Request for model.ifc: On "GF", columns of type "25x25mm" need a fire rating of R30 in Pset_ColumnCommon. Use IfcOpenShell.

First a look at what the model holds.

```python
import ifcopenshell
import ifcopenshell.util.element

model = ifcopenshell.open("model.ifc")
print(model.schema)
storey = next(s for s in model.by_type("IfcBuildingStorey") if s.Name == "GF")
columns = [e for e in ifcopenshell.util.element.get_decomposition(storey) if e.is_a("IfcColumn")]
seen = {}
for e in columns:
    element_type = ifcopenshell.util.element.get_type(e)
    key = (element_type.Name if element_type != e and element_type else None, ifcopenshell.util.element.get_pset(e, "Pset_ColumnCommon", "FireRating"))
    seen[key] = seen.get(key, 0) + 1
for (name, value), count in sorted(seen.items(), key=str):
    print(count, "x", name, "|", value)
```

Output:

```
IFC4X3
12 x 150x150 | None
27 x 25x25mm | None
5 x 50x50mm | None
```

```python
import ifcopenshell
import ifcopenshell.api.pset
import ifcopenshell.util.element

model = ifcopenshell.open("model.ifc")

storey = next(s for s in model.by_type("IfcBuildingStorey") if s.Name == "GF")
columns = [e for e in ifcopenshell.util.element.get_decomposition(storey) if e.is_a("IfcColumn")]

count = 0
for e in columns:
    element_type = ifcopenshell.util.element.get_type(e)
    if element_type in (None, e) or element_type.Name != "25x25mm":
        continue
    # add_pset returns the element's existing set when there is one.
    pset = ifcopenshell.api.pset.add_pset(model, product=e, name="Pset_ColumnCommon")
    ifcopenshell.api.pset.edit_pset(model, pset=pset, properties={"FireRating": "R30"})
    count += 1

print(count, "columns updated")

model.write("model_rev.ifc")
```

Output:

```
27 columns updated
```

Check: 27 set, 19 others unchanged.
